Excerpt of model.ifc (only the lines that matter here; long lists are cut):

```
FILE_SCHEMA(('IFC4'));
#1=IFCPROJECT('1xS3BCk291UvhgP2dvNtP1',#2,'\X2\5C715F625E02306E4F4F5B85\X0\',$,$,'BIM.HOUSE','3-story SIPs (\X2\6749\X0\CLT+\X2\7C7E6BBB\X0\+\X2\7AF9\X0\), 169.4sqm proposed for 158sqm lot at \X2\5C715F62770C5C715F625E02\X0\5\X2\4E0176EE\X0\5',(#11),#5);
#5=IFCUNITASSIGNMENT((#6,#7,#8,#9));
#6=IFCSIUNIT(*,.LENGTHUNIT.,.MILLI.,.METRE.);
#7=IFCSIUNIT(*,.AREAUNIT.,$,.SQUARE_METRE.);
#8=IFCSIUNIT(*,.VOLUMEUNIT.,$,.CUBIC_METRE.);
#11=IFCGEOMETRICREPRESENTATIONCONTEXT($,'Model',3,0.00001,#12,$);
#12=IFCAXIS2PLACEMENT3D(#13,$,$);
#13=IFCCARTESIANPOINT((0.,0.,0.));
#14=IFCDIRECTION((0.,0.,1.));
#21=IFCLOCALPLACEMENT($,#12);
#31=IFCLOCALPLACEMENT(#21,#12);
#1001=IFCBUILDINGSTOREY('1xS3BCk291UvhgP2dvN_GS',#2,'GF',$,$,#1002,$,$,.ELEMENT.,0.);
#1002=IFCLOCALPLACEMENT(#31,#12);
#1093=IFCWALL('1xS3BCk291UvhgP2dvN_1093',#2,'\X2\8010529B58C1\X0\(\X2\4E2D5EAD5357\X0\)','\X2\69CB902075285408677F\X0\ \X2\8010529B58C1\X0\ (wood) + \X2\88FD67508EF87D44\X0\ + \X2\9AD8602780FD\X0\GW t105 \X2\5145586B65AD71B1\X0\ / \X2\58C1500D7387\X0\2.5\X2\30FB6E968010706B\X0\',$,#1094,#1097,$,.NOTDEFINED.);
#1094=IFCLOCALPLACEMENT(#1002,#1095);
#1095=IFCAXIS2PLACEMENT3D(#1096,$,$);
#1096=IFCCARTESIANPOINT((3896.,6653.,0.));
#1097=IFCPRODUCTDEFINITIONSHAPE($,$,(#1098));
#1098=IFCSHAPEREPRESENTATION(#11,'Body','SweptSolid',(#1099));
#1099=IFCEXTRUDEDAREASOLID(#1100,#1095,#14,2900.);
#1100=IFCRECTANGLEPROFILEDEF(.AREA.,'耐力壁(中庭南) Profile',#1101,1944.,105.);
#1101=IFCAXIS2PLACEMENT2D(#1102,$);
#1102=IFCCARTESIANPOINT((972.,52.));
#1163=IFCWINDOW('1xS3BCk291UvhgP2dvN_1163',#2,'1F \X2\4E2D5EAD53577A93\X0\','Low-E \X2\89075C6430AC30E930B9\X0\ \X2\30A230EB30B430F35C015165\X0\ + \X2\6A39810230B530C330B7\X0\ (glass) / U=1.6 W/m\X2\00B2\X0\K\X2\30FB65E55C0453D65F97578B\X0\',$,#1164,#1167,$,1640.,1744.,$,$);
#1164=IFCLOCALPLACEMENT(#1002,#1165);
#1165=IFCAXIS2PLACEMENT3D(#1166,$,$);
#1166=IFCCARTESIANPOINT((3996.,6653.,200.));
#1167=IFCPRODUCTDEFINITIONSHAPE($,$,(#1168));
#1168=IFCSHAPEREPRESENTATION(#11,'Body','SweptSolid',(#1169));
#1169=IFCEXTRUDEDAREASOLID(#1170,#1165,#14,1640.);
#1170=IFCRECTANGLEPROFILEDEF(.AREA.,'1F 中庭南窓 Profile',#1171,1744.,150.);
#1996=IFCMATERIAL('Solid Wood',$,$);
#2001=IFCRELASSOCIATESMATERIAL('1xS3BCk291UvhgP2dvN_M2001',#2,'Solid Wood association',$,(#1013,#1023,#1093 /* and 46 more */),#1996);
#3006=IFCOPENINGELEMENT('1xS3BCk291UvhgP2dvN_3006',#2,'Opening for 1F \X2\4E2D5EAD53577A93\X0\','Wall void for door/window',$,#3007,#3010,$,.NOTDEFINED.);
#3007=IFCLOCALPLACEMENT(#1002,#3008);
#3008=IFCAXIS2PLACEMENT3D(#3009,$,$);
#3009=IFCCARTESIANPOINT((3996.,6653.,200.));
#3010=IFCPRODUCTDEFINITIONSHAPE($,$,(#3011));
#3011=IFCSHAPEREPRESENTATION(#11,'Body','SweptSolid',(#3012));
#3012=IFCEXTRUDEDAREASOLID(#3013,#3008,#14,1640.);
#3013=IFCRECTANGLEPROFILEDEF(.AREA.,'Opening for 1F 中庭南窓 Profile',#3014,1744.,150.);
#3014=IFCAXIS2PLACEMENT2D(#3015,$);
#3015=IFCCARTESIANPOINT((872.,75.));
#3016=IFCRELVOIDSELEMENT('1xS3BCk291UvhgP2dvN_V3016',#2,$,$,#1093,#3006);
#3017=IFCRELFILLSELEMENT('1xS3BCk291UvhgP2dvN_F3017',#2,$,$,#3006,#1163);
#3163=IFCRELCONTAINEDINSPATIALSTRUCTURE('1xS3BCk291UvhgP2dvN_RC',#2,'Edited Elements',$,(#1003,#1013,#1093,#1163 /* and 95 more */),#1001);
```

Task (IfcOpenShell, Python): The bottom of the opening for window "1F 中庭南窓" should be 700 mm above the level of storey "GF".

```python
import numpy as np
import ifcopenshell
import ifcopenshell.api.geometry
import ifcopenshell.geom
import ifcopenshell.util.element
import ifcopenshell.util.placement
import ifcopenshell.util.shape
import ifcopenshell.util.unit

model = ifcopenshell.open("model.ifc")
unit_scale = ifcopenshell.util.unit.calculate_unit_scale(model)

window = model.by_guid("1xS3BCk291UvhgP2dvN_1163")
opening = window.FillsVoids[0].RelatingOpeningElement
storey = ifcopenshell.util.element.get_container(window, ifc_class="IfcBuildingStorey")
level = ifcopenshell.util.placement.get_local_placement(storey.ObjectPlacement)[2, 3]

# The opening's origin need not be at the sill, so measure its lowest point.
shape = ifcopenshell.geom.create_shape(ifcopenshell.geom.settings(), opening)
bottom = ifcopenshell.util.shape.get_shape_bottom_elevation(shape, shape.geometry) / unit_scale
dz = level + 0.7 / unit_scale - bottom

shift = np.array([0.0, 0.0, dz])
# The window is not placed relative to its opening, so move both.
for product in (opening, window):
    matrix = ifcopenshell.util.placement.get_local_placement(product.ObjectPlacement)
    matrix[:3, 3] += shift
    ifcopenshell.api.geometry.edit_object_placement(model, product=product, matrix=matrix, is_si=False)

print(f"moved by {dz * unit_scale:+.3f} m")

model.write("model-out.ifc")
```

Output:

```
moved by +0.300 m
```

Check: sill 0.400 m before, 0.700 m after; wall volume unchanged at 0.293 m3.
